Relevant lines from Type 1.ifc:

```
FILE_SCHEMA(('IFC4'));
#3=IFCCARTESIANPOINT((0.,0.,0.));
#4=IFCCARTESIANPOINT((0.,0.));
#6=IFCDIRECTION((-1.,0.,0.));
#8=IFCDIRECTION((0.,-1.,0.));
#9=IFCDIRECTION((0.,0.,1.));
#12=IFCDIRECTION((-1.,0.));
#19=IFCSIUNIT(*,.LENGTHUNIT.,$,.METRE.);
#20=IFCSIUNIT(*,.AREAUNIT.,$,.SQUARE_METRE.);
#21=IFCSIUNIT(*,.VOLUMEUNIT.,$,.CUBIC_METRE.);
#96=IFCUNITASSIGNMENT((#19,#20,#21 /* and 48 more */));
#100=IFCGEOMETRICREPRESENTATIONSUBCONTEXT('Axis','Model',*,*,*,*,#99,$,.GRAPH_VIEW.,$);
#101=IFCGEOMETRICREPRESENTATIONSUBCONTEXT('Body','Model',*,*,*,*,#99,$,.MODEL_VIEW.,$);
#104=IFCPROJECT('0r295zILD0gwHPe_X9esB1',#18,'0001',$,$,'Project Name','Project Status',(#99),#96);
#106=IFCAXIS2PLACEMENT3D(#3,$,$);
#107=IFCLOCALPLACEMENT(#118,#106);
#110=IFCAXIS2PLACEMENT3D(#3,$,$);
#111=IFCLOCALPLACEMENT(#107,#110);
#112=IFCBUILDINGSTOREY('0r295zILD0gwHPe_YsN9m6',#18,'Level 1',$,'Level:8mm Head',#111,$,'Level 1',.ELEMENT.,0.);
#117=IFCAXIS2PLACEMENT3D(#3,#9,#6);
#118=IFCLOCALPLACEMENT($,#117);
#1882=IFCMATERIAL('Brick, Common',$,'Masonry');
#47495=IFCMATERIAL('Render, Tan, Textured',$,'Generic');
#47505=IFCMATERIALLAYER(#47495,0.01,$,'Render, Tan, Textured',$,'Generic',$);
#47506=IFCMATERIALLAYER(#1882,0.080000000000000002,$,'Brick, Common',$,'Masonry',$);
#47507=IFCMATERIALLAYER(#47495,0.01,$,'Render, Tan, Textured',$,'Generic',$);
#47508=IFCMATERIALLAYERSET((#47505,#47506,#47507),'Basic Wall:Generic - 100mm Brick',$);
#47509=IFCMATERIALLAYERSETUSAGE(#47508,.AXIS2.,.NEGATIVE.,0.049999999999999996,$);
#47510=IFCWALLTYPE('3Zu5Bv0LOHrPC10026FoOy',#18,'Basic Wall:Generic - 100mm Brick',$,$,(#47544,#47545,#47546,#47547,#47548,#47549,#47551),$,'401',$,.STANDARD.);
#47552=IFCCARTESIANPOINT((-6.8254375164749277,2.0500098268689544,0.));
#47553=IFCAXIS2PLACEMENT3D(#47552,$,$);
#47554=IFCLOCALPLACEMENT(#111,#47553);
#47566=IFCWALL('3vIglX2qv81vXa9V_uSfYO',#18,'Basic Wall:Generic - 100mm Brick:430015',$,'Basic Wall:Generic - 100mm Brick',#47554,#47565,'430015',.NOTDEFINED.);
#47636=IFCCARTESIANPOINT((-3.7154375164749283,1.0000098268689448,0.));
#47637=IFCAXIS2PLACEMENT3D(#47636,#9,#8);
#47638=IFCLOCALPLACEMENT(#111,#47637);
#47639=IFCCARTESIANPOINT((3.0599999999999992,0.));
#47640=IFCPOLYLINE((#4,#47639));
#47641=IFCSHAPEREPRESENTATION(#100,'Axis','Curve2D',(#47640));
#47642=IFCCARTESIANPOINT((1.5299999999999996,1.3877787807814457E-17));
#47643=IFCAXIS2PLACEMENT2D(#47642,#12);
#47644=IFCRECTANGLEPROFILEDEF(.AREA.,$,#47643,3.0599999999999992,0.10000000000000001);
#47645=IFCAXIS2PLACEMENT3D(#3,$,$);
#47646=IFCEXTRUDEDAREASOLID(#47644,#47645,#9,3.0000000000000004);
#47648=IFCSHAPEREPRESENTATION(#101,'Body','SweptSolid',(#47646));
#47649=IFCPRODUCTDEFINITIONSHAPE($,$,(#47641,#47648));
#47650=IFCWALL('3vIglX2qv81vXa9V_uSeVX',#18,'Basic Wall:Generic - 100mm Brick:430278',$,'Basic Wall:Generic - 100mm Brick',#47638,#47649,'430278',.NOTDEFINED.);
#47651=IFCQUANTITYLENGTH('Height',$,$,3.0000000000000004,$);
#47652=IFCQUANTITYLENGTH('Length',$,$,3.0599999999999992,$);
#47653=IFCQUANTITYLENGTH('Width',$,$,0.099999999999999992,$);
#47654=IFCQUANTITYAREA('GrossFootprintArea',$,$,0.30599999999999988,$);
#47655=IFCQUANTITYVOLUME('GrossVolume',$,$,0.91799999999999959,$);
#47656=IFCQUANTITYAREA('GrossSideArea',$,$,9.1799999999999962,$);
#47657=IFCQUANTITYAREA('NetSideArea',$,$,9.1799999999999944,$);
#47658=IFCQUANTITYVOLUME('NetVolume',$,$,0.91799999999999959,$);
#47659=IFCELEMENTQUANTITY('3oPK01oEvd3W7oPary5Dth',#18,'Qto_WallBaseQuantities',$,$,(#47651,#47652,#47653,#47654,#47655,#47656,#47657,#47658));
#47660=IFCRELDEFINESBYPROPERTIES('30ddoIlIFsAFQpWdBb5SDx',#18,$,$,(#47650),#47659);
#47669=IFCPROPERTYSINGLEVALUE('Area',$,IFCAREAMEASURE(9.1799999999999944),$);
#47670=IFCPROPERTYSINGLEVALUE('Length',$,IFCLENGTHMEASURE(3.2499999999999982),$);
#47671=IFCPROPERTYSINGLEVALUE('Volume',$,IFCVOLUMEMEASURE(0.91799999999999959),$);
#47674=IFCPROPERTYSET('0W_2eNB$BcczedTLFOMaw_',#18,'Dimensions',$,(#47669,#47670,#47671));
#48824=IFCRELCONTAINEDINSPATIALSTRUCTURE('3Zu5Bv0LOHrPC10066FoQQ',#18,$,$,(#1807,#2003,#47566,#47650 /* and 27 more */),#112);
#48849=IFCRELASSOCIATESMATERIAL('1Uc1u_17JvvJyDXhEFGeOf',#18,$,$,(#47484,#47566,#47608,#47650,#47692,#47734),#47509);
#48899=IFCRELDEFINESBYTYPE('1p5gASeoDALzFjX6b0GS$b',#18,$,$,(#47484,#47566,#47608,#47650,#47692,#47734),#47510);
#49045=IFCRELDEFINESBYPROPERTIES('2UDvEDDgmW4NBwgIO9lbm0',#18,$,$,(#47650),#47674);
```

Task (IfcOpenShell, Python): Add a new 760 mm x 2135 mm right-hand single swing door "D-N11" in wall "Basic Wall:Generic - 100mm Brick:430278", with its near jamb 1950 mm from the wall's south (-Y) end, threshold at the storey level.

```python
import numpy as np
import ifcopenshell
import ifcopenshell.api.feature
import ifcopenshell.api.geometry
import ifcopenshell.api.pset
import ifcopenshell.api.root
import ifcopenshell.api.spatial
import ifcopenshell.geom
import ifcopenshell.util.element
import ifcopenshell.util.placement
import ifcopenshell.util.representation
import ifcopenshell.util.shape
import ifcopenshell.util.unit

model = ifcopenshell.open("Type 1.ifc")
unit_scale = ifcopenshell.util.unit.calculate_unit_scale(model)
area_scale = ifcopenshell.util.unit.calculate_unit_scale(model, "AREAUNIT")
volume_scale = ifcopenshell.util.unit.calculate_unit_scale(model, "VOLUMEUNIT")
settings = ifcopenshell.geom.settings()


def volume(element):
    """Net volume in cubic metres, openings subtracted."""
    shape = ifcopenshell.geom.create_shape(settings, element)
    return ifcopenshell.util.shape.get_volume(shape.geometry)


wall = model.by_guid("3vIglX2qv81vXa9V_uSeVX")
storey = ifcopenshell.util.element.get_container(wall, ifc_class="IfcBuildingStorey")
context = ifcopenshell.util.representation.get_context(model, "Model", "Body", "MODEL_VIEW")
before = volume(wall)

width, height, from_end, sill = 0.76, 2.135, 1.95, 0.0  # metres

# The wall runs along its own X axis, and the end named is its -X end.
wall_shape = ifcopenshell.geom.create_shape(settings, wall)
x, y, z = ifcopenshell.util.shape.get_vertices(wall_shape.geometry).T
start = x.min() + from_end
face, thickness = float(y.min()), float(y.max() - y.min())
wall_matrix = ifcopenshell.util.placement.get_local_placement(wall.ObjectPlacement)
level = ifcopenshell.util.placement.get_local_placement(storey.ObjectPlacement)[2, 3]


def in_wall(x, y):
    """Placement at x, y metres in the wall's axes, at sill height."""
    matrix = wall_matrix.copy()
    matrix[:, 3] = wall_matrix @ np.array([x / unit_scale, y / unit_scale, 0.0, 1.0])
    matrix[2, 3] = level + sill / unit_scale
    return matrix


# Opening: a box that overshoots both wall faces by 50 mm.
opening = ifcopenshell.api.root.create_entity(model, ifc_class="IfcOpeningElement", predefined_type="OPENING")
box = ifcopenshell.api.geometry.add_wall_representation(
    model, context=context, length=width, height=height, thickness=thickness + 0.1
)
ifcopenshell.api.geometry.assign_representation(model, product=opening, representation=box)
ifcopenshell.api.geometry.edit_object_placement(model, product=opening, matrix=in_wall(start, face - 0.05), is_si=False)
ifcopenshell.api.feature.add_feature(model, feature=opening, element=wall)

door = ifcopenshell.api.root.create_entity(model, ifc_class="IfcDoor", name="D-N11", predefined_type="DOOR")
door.OverallWidth, door.OverallHeight = width / unit_scale, height / unit_scale
door.OperationType = "SINGLE_SWING_RIGHT"
body = ifcopenshell.api.geometry.add_door_representation(
    model,
    context=context,
    overall_width=door.OverallWidth,
    overall_height=door.OverallHeight,
    operation_type="SINGLE_SWING_RIGHT",
    lining_properties={"LiningDepth": thickness / unit_scale, "ThresholdDepth": thickness / unit_scale},
)
ifcopenshell.api.geometry.assign_representation(model, product=door, representation=body)
ifcopenshell.api.spatial.assign_container(model, products=[door], relating_structure=storey)
ifcopenshell.api.feature.add_filling(model, opening=opening, element=door)

# The lining spans the wall, so the door starts at the wall face.
ifcopenshell.api.geometry.edit_object_placement(model, product=door, matrix=in_wall(start, face), is_si=False)

after = volume(wall)

# Update the wall's stored quantities.
qto = model.by_id(ifcopenshell.util.element.get_pset(wall, "Qto_WallBaseQuantities", should_inherit=False)["id"])
ifcopenshell.api.pset.edit_qto(model, qto=qto, properties={
    "NetSideArea": after / thickness / area_scale,
    "NetVolume": after / volume_scale,
})
pset = model.by_id(ifcopenshell.util.element.get_pset(wall, "Dimensions", should_inherit=False)["id"])
ifcopenshell.api.pset.edit_pset(model, pset=pset, properties={
    "Area": model.create_entity("IfcAreaMeasure", after / thickness / area_scale),
    "Volume": model.create_entity("IfcVolumeMeasure", after / volume_scale),
})

print(f"wall volume {before:.3f} -> {after:.3f} m3")

model.write("Type 1_rev.ifc")
```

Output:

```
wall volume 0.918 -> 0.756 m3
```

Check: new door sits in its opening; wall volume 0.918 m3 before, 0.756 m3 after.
